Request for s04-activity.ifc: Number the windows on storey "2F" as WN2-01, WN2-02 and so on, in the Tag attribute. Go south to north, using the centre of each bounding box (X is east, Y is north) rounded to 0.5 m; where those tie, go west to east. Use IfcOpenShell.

First a look at what the model holds.

```python
import ifcopenshell
import ifcopenshell.util.element
import ifcopenshell.util.placement

model = ifcopenshell.open("s04-activity.ifc")
print(model.schema)
storey = next(s for s in model.by_type("IfcBuildingStorey") if s.Name == "2F")
windows = [e for e in ifcopenshell.util.element.get_decomposition(storey) if e.is_a("IfcWindow")]
for e in sorted(windows, key=lambda e: e.id()):
    origin = ifcopenshell.util.placement.get_local_placement(e.ObjectPlacement)[:3, 3]
    print(e.id(), e.Tag, e.Name, origin.round(2) + 0.0, sep=" | ")
```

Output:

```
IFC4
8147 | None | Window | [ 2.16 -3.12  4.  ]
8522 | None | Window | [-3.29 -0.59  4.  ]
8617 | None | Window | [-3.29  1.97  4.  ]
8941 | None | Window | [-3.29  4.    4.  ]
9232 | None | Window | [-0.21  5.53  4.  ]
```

```python
import ifcopenshell
import ifcopenshell.geom
import ifcopenshell.util.element
import ifcopenshell.util.shape

model = ifcopenshell.open("s04-activity.ifc")
settings = ifcopenshell.geom.settings()
settings.set("use-world-coords", True)


def centre(element):
    shape = ifcopenshell.geom.create_shape(settings, element)
    return ifcopenshell.util.shape.get_bbox_centroid(shape.geometry)


storey = next(s for s in model.by_type("IfcBuildingStorey") if s.Name == "2F")
windows = [e for e in ifcopenshell.util.element.get_decomposition(storey) if e.is_a("IfcWindow")]

# Insertion points can sit at a corner or the storey origin, so sort by the geometry (in metres).
centres = {e: centre(e) for e in windows}
windows.sort(key=lambda e: (round(centres[e][1] / 0.5), centres[e][0]))

for i, e in enumerate(windows, start=1):
    number = f"WN2-{i:02d}"
    e.Tag = number
    print(e.id(), number)

model.write("s04-activity_updated.ifc")
```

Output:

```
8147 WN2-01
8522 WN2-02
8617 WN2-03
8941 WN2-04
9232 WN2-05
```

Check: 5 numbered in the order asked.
